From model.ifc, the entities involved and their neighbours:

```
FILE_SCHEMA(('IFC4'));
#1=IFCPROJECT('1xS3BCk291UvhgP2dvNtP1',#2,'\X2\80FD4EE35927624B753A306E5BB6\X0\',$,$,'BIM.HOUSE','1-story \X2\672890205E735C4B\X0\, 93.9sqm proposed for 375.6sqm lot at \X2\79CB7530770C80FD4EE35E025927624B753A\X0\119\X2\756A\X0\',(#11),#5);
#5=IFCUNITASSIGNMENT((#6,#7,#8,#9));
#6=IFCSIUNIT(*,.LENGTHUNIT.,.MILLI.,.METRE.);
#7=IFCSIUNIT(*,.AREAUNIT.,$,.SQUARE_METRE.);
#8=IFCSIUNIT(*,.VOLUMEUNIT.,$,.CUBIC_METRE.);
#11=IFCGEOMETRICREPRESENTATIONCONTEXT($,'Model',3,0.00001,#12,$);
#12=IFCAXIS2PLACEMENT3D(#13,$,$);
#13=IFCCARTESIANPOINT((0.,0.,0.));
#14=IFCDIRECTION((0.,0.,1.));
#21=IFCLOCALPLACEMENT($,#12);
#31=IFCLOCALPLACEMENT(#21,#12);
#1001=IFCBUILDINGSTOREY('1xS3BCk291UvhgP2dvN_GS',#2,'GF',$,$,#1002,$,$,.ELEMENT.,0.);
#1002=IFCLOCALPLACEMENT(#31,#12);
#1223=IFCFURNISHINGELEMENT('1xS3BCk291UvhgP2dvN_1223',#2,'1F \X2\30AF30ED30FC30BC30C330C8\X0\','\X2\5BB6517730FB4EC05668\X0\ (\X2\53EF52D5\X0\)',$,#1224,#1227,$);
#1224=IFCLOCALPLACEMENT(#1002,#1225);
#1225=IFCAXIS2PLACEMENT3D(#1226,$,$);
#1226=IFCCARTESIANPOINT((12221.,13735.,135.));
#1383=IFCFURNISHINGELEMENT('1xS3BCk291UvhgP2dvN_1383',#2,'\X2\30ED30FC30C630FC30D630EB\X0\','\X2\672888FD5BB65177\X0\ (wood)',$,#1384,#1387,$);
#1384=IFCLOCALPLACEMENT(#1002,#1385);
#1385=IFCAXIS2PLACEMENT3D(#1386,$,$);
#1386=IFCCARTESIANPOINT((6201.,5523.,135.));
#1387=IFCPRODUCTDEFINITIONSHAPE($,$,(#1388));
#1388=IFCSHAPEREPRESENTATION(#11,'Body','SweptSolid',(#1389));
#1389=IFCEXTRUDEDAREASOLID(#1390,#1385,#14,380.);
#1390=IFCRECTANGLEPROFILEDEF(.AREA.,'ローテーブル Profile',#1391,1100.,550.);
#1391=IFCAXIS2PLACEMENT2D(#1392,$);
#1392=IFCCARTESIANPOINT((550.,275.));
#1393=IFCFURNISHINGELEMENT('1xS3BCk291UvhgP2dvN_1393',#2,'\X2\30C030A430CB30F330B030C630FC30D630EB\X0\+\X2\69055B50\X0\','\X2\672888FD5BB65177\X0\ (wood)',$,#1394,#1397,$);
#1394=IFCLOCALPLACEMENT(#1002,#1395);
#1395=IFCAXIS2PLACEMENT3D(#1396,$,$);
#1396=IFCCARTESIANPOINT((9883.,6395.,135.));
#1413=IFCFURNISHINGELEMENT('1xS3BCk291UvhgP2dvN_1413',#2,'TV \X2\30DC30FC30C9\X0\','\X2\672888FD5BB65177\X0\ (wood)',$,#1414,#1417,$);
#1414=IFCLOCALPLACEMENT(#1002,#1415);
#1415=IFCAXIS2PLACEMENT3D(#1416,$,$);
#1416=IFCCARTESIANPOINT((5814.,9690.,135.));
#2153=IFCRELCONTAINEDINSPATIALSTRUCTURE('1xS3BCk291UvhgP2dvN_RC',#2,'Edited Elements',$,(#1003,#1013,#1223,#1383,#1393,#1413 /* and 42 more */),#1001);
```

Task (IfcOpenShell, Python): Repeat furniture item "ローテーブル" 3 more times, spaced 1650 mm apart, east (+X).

```python
import numpy as np
import ifcopenshell
import ifcopenshell.api.geometry
import ifcopenshell.api.root
import ifcopenshell.util.element
import ifcopenshell.util.placement

model = ifcopenshell.open("model.ifc")


def reuse_history(source, copy):
    """copy_class also copies each property set's owner history, people and application; keep the originals."""
    for rel in copy.IsDefinedBy:
        if rel.is_a("IfcRelDefinesByProperties") and (history := rel.RelatingPropertyDefinition.OwnerHistory):
            rel.RelatingPropertyDefinition.OwnerHistory = source.OwnerHistory
            ifcopenshell.util.element.remove_deep2(model, history)


source = model.by_guid("1xS3BCk291UvhgP2dvN_1383")
base = ifcopenshell.util.placement.get_local_placement(source.ObjectPlacement)
step = np.array([1.0, 0.0, 0.0]) * 1650.0

for i in range(1, 4):
    copy = ifcopenshell.api.root.copy_class(model, product=source)
    copy.Representation = ifcopenshell.util.element.copy_deep(
        model, source.Representation, exclude=["IfcGeometricRepresentationContext", "IfcRepresentationMap"]
    )
    reuse_history(source, copy)
    matrix = base.copy()
    matrix[:3, 3] += i * step
    print("added at", matrix[:3, 3].round(3) + 0.0)
    ifcopenshell.api.geometry.edit_object_placement(model, product=copy, matrix=matrix, is_si=False)

model.write("model-out.ifc")
```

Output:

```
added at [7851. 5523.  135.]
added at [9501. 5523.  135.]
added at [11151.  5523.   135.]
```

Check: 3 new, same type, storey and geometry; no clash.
